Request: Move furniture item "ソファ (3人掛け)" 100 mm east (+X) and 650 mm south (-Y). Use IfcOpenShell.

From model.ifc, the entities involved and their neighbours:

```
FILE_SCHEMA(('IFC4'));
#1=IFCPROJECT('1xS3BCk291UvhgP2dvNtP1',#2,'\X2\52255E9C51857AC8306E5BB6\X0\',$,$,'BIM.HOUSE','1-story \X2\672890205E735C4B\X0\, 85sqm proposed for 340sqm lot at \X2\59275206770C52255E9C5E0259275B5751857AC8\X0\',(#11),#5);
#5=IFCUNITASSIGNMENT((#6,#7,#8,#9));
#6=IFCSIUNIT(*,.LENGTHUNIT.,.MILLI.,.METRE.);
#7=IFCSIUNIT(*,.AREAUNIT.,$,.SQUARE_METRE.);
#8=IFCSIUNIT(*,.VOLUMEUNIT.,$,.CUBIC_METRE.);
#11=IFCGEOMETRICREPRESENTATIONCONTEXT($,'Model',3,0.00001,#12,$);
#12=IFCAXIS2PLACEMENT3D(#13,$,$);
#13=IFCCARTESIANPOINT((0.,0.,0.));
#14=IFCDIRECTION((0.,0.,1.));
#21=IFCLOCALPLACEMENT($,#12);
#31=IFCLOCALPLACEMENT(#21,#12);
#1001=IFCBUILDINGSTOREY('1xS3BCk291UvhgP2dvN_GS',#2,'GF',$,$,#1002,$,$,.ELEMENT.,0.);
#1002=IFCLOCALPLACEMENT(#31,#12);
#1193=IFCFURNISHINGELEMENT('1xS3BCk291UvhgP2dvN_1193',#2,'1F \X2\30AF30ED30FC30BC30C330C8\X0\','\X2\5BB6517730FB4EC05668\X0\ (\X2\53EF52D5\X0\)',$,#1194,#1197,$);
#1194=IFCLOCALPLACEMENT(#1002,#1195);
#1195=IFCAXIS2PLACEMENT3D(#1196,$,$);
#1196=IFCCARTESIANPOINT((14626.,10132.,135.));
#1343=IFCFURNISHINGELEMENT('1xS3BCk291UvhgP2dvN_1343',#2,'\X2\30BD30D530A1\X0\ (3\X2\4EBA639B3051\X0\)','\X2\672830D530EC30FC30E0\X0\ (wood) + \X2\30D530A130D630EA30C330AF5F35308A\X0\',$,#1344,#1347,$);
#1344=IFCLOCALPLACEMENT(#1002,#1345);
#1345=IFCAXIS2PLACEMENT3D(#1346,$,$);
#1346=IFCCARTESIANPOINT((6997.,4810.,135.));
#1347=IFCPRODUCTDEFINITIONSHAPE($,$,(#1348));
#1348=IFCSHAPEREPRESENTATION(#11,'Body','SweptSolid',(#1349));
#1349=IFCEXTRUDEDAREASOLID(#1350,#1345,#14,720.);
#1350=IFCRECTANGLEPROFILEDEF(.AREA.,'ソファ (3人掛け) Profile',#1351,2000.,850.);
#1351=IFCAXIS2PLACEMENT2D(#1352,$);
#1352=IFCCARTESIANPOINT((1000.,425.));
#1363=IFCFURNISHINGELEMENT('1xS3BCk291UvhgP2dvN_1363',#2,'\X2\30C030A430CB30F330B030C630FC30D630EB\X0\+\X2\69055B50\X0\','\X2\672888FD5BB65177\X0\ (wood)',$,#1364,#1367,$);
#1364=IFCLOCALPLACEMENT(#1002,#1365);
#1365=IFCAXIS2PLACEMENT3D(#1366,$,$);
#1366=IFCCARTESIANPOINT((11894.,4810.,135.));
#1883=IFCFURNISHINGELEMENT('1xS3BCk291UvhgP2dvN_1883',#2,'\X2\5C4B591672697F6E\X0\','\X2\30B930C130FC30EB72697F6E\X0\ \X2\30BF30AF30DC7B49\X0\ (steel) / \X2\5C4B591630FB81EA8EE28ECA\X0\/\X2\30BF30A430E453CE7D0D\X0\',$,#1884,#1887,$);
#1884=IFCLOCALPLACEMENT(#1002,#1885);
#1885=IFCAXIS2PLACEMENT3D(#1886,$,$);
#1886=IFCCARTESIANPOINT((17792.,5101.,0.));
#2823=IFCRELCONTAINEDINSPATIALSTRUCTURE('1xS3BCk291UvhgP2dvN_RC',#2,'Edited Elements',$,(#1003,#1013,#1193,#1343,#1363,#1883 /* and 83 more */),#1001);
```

```python
import ifcopenshell
import ifcopenshell.api.geometry
import ifcopenshell.util.placement

model = ifcopenshell.open("model.ifc")

item = model.by_guid("1xS3BCk291UvhgP2dvN_1343")
matrix = ifcopenshell.util.placement.get_local_placement(item.ObjectPlacement)
matrix[0, 3] += 100.0
matrix[1, 3] -= 650.0
ifcopenshell.api.geometry.edit_object_placement(model, product=item, matrix=matrix, is_si=False)

print(ifcopenshell.util.placement.get_local_placement(item.ObjectPlacement).round(3) + 0.0)

model.write("model-out.ifc")
```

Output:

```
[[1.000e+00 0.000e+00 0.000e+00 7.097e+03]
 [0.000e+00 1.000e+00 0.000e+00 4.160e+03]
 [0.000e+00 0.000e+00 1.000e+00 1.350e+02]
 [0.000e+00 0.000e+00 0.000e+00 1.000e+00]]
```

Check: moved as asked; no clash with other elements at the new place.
